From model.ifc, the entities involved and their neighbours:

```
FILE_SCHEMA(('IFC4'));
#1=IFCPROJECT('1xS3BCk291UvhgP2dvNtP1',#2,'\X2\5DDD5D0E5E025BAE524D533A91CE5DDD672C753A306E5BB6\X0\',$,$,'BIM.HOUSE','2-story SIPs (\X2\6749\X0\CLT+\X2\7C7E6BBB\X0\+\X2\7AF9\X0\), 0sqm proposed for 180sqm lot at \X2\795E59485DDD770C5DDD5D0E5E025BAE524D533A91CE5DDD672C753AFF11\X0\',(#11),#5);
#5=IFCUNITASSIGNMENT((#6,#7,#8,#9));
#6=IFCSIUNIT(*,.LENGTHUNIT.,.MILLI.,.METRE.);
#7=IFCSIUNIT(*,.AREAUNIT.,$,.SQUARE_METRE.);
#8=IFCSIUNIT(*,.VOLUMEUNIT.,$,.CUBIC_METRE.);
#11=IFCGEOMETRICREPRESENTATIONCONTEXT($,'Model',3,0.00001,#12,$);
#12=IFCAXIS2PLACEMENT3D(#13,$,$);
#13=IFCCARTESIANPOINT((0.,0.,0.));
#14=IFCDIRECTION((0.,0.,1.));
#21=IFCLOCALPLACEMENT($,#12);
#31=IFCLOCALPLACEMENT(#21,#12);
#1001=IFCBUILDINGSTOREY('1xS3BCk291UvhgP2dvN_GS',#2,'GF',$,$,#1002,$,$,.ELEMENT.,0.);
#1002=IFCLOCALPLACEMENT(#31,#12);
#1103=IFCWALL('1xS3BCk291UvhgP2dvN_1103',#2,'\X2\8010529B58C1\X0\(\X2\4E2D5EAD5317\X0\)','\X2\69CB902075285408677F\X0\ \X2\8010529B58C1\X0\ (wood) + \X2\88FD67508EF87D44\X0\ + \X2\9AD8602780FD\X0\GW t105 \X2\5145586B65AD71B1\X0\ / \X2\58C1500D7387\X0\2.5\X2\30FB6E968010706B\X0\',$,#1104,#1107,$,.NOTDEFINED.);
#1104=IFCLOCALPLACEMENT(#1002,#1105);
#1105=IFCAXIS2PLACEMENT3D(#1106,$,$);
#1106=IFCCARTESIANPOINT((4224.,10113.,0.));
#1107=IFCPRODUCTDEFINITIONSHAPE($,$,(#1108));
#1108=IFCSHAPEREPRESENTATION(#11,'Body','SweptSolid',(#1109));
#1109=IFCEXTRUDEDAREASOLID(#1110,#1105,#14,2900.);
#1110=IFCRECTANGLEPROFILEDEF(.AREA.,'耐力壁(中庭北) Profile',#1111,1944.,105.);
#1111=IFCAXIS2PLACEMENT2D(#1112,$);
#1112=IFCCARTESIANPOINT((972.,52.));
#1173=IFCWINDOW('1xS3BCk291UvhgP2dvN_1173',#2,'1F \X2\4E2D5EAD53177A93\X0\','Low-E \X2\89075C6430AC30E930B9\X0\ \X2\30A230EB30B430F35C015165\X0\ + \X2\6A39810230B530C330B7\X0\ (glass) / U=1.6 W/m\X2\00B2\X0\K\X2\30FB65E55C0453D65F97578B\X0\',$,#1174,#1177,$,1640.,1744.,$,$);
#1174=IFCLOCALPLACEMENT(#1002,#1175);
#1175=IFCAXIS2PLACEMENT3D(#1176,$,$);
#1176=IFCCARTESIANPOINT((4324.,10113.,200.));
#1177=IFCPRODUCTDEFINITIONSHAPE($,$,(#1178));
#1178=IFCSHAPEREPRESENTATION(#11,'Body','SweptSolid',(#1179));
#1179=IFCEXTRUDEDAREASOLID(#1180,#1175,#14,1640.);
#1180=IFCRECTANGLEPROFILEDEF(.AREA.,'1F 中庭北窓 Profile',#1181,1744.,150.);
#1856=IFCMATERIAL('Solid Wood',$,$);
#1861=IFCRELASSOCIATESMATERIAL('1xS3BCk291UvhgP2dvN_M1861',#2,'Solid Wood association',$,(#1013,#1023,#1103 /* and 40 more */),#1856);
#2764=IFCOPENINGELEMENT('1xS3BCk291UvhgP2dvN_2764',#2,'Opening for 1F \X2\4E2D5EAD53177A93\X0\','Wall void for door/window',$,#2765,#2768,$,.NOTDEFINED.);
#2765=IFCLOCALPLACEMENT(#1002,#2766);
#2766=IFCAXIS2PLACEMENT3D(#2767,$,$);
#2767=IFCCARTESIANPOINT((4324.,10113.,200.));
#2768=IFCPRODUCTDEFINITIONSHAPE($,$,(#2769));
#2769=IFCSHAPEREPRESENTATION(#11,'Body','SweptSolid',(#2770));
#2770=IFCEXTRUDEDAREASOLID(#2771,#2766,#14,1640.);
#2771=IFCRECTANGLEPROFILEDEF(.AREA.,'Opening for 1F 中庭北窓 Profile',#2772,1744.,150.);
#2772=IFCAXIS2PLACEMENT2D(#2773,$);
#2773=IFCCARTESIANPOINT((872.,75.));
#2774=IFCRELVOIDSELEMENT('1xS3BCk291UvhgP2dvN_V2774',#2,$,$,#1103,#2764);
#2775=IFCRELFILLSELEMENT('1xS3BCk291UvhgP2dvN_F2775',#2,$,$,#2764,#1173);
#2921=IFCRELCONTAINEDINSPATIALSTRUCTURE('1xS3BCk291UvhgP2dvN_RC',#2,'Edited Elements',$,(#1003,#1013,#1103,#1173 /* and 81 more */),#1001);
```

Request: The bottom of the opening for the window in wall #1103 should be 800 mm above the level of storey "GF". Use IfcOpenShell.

```python
import numpy as np
import ifcopenshell
import ifcopenshell.api.geometry
import ifcopenshell.geom
import ifcopenshell.util.element
import ifcopenshell.util.placement
import ifcopenshell.util.shape
import ifcopenshell.util.unit

model = ifcopenshell.open("model.ifc")
unit_scale = ifcopenshell.util.unit.calculate_unit_scale(model)

window = model.by_guid("1xS3BCk291UvhgP2dvN_1173")
opening = window.FillsVoids[0].RelatingOpeningElement
storey = ifcopenshell.util.element.get_container(window, ifc_class="IfcBuildingStorey")
level = ifcopenshell.util.placement.get_local_placement(storey.ObjectPlacement)[2, 3]

# The opening's origin need not be at the sill, so measure its lowest point.
shape = ifcopenshell.geom.create_shape(ifcopenshell.geom.settings(), opening)
bottom = ifcopenshell.util.shape.get_shape_bottom_elevation(shape, shape.geometry) / unit_scale
dz = level + 0.8 / unit_scale - bottom

shift = np.array([0.0, 0.0, dz])
# The window is not placed relative to its opening, so move both.
for product in (opening, window):
    matrix = ifcopenshell.util.placement.get_local_placement(product.ObjectPlacement)
    matrix[:3, 3] += shift
    ifcopenshell.api.geometry.edit_object_placement(model, product=product, matrix=matrix, is_si=False)

print(f"moved by {dz * unit_scale:+.3f} m")

model.write("model_rev.ifc")
```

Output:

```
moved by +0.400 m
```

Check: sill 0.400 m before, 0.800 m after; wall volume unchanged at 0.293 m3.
